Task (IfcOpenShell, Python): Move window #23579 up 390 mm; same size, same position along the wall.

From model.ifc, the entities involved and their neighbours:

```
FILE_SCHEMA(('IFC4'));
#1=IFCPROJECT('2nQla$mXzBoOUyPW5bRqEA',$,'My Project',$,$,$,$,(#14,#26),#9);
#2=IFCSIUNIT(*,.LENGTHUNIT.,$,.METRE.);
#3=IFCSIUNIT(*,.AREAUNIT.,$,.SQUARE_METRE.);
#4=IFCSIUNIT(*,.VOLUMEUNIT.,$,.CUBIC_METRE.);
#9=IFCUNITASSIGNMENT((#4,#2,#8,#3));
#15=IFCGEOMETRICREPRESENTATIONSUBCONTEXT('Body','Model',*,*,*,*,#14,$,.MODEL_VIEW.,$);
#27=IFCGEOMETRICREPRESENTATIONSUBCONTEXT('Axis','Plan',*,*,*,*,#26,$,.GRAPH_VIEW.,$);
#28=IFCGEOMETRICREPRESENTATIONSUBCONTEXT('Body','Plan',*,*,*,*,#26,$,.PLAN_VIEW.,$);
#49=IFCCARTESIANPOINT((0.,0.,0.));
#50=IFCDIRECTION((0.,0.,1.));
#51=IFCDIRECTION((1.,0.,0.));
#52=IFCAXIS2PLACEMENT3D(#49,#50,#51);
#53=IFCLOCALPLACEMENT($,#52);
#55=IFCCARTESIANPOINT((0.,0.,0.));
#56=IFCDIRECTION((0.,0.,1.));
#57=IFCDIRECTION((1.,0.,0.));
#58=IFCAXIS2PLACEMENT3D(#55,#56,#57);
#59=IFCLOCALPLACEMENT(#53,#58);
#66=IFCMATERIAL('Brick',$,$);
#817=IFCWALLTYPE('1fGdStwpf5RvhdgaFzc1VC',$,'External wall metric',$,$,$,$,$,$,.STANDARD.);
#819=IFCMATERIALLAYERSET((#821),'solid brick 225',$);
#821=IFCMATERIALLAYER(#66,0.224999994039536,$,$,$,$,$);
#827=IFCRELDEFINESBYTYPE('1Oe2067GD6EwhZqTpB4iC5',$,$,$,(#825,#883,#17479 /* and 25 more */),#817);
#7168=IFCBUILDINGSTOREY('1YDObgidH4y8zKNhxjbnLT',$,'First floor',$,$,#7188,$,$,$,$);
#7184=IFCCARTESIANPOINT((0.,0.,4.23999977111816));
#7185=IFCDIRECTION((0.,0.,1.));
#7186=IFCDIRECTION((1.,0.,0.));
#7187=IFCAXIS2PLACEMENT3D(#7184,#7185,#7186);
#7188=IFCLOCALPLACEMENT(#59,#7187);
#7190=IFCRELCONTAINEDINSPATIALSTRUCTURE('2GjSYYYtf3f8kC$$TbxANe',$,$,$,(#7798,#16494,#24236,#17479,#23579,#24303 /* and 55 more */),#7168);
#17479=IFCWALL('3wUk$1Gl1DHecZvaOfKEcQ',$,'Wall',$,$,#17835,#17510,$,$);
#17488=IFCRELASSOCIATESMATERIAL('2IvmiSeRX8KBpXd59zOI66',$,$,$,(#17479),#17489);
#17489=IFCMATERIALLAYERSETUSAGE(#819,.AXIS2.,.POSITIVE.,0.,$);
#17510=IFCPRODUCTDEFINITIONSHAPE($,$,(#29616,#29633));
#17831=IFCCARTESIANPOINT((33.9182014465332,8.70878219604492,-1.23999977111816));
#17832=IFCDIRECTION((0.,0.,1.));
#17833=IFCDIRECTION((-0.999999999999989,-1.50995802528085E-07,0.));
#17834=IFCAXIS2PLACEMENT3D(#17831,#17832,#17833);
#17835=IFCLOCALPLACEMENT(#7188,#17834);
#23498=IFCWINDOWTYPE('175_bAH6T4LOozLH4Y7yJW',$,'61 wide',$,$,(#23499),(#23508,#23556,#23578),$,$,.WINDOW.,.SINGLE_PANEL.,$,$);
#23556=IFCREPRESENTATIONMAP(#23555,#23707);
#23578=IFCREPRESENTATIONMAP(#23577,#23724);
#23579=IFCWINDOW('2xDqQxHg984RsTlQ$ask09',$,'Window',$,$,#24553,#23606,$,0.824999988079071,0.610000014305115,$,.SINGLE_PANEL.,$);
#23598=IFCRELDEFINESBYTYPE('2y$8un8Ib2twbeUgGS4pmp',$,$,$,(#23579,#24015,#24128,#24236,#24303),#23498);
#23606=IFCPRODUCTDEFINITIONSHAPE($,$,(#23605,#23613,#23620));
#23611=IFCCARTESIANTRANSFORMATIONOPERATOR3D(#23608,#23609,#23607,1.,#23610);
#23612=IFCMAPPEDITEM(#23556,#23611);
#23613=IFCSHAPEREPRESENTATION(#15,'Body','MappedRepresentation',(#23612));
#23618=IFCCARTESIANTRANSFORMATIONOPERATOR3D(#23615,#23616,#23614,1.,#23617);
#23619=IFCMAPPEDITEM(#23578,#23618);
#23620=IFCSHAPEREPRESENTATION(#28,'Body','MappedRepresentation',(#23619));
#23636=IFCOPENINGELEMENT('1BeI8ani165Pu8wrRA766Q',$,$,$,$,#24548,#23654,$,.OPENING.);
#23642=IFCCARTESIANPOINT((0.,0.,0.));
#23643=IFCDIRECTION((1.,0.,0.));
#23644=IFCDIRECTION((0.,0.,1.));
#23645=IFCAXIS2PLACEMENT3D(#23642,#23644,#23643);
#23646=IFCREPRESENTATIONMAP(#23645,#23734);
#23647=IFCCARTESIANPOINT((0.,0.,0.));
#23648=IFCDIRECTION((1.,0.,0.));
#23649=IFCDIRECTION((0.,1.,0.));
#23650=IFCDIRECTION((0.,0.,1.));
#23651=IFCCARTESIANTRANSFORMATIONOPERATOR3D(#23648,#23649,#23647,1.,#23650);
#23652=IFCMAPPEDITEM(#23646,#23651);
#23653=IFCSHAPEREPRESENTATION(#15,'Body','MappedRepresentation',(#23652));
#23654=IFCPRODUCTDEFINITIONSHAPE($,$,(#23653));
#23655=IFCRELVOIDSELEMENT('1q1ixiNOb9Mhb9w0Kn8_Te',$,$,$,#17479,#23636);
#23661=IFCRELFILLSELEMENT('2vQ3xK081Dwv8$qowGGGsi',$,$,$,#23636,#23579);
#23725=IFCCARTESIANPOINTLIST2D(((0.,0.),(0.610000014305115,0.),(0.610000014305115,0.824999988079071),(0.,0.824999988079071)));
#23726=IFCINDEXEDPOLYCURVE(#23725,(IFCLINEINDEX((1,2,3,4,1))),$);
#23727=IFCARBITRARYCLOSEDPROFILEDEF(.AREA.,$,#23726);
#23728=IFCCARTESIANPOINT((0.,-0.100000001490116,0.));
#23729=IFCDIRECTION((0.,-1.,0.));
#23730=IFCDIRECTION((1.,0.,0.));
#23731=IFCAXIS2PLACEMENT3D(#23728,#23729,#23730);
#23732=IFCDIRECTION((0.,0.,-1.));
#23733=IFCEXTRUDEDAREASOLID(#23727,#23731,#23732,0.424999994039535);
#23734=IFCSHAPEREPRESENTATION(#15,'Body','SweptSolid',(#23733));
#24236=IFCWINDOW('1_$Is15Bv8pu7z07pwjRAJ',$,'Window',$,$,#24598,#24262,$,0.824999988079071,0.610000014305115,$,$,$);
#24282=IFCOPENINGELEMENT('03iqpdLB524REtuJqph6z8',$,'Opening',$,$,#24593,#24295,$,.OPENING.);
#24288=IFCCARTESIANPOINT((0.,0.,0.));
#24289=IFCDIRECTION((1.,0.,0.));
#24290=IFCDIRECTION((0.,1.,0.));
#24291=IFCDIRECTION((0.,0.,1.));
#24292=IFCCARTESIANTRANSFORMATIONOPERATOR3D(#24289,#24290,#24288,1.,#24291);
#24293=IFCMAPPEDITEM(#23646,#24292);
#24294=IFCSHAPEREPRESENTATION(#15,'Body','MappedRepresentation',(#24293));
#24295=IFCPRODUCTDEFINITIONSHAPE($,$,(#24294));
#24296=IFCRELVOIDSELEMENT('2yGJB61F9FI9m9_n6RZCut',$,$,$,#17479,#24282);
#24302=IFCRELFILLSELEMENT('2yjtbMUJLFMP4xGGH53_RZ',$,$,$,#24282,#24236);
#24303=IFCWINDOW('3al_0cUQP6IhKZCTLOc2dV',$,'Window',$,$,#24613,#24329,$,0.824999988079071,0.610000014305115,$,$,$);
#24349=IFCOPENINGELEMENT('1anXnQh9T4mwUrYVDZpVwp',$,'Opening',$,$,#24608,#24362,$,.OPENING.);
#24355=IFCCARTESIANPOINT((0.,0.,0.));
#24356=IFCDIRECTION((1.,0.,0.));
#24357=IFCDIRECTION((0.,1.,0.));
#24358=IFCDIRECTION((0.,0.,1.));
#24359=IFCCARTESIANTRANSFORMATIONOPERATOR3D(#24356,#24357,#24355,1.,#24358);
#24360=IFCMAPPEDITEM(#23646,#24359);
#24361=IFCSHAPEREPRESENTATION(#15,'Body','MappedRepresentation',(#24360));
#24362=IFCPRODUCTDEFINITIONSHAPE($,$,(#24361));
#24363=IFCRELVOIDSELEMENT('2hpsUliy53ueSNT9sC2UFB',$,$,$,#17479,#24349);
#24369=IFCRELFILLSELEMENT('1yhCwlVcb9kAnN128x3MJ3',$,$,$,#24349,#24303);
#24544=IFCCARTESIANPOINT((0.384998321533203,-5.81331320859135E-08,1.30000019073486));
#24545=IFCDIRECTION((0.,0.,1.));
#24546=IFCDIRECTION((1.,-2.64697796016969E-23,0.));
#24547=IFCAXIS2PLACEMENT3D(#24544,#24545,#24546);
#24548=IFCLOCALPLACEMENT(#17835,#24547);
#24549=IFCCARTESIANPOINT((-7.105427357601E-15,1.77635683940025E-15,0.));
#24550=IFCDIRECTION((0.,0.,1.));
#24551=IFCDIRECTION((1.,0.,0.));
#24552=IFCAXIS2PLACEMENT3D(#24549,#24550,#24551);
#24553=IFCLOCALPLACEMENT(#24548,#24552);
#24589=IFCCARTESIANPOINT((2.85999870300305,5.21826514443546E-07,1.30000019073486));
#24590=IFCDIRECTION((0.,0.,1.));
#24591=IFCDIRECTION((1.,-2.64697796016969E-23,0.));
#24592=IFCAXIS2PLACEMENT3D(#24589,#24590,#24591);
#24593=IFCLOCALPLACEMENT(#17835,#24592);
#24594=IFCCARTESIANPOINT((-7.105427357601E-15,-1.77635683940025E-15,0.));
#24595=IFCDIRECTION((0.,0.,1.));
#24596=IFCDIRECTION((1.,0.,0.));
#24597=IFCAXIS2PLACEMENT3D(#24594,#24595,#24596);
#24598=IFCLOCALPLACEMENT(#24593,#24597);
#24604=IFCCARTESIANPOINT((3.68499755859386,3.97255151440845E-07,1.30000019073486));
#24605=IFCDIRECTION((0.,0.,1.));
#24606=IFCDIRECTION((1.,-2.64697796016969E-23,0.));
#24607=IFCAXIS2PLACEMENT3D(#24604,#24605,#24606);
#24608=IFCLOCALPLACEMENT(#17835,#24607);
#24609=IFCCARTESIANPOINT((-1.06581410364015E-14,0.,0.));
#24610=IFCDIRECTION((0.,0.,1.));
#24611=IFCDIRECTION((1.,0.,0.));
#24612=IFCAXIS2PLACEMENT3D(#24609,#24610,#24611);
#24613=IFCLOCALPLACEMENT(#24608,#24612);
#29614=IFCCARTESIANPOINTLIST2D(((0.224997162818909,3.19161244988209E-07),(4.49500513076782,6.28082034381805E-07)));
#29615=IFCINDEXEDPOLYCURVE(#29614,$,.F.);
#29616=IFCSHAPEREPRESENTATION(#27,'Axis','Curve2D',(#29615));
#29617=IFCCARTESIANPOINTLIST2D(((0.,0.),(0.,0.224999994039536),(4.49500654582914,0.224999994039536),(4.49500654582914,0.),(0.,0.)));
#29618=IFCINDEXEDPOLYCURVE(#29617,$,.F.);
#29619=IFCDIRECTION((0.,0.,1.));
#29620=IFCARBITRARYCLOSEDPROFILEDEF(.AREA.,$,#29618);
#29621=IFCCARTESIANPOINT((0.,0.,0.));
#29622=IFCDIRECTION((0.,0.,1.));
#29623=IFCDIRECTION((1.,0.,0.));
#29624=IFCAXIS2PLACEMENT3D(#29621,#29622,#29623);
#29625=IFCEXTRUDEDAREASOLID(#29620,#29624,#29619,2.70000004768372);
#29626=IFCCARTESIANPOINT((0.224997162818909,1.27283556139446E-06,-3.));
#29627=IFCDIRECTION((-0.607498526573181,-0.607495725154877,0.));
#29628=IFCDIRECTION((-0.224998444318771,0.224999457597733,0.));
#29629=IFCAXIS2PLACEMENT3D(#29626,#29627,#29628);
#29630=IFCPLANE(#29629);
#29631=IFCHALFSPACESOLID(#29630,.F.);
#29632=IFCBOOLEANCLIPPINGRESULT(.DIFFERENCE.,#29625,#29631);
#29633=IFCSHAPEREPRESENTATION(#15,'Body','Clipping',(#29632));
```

```python
import numpy as np
import ifcopenshell
import ifcopenshell.api.geometry
import ifcopenshell.util.placement
import ifcopenshell.util.unit

model = ifcopenshell.open("model.ifc")
unit_scale = ifcopenshell.util.unit.calculate_unit_scale(model)

window = model.by_id(23579)
opening = window.FillsVoids[0].RelatingOpeningElement
dz = 0.39

shift = np.array([0.0, 0.0, dz])
# The window is placed relative to its opening, so it follows when the opening moves.
matrix = ifcopenshell.util.placement.get_local_placement(opening.ObjectPlacement)
matrix[:3, 3] += shift
ifcopenshell.api.geometry.edit_object_placement(
    model, product=opening, matrix=matrix, is_si=False, should_transform_children=True
)

print(f"moved by {dz * unit_scale:+.3f} m")

model.write("model_edited.ifc")
```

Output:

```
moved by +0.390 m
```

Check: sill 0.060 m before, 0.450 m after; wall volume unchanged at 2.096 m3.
